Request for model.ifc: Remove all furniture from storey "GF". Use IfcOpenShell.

First a look at what the model holds.

```python
import ifcopenshell
import ifcopenshell.util.element

model = ifcopenshell.open("model.ifc")
print(model.schema)
storey = next(s for s in model.by_type("IfcBuildingStorey") if s.Name == "GF")
furniture = [e for e in ifcopenshell.util.element.get_decomposition(storey) if e.is_a("IfcFurnishingElement")]
seen = {}
for e in furniture:
    element_type = ifcopenshell.util.element.get_type(e)
    name = element_type.Name if element_type not in (None, e) else None
    seen[name] = seen.get(name, 0) + 1
for name, count in sorted(seen.items(), key=str):
    print(count, "x", name)
```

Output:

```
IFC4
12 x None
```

```python
import ifcopenshell
import ifcopenshell.api.root
import ifcopenshell.util.element

model = ifcopenshell.open("model.ifc")

storey = next(s for s in model.by_type("IfcBuildingStorey") if s.Name == "GF")
furniture = [e for e in ifcopenshell.util.element.get_decomposition(storey) if e.is_a("IfcFurnishingElement")]

for e in furniture:
    ifcopenshell.api.root.remove_product(model, product=e)
print(len(furniture), "removed")

model.write("model_rev.ifc")
```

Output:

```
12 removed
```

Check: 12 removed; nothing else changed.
